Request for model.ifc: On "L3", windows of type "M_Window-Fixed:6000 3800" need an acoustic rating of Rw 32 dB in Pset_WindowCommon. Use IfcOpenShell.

First a look at what the model holds.

```python
import ifcopenshell
import ifcopenshell.util.element

model = ifcopenshell.open("model.ifc")
print(model.schema)
storey = next(s for s in model.by_type("IfcBuildingStorey") if s.Name == "L3")
windows = [e for e in ifcopenshell.util.element.get_decomposition(storey) if e.is_a("IfcWindow")]
seen = {}
for e in windows:
    element_type = ifcopenshell.util.element.get_type(e)
    key = (element_type.Name if element_type != e and element_type else None, ifcopenshell.util.element.get_pset(e, "Pset_WindowCommon", "AcousticRating"))
    seen[key] = seen.get(key, 0) + 1
for (name, value), count in sorted(seen.items(), key=str):
    print(count, "x", name, "|", value)
```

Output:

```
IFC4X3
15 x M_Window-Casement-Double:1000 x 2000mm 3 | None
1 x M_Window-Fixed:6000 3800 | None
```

```python
import ifcopenshell
import ifcopenshell.api.pset
import ifcopenshell.util.element

model = ifcopenshell.open("model.ifc")

storey = next(s for s in model.by_type("IfcBuildingStorey") if s.Name == "L3")
windows = [e for e in ifcopenshell.util.element.get_decomposition(storey) if e.is_a("IfcWindow")]

count = 0
for e in windows:
    element_type = ifcopenshell.util.element.get_type(e)
    if element_type in (None, e) or element_type.Name != "M_Window-Fixed:6000 3800":
        continue
    # add_pset returns the element's existing set when there is one.
    pset = ifcopenshell.api.pset.add_pset(model, product=e, name="Pset_WindowCommon")
    ifcopenshell.api.pset.edit_pset(model, pset=pset, properties={"AcousticRating": "Rw 32 dB"})
    count += 1

print(count, "windows updated")

model.write("model_edited.ifc")
```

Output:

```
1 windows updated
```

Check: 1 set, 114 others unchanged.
